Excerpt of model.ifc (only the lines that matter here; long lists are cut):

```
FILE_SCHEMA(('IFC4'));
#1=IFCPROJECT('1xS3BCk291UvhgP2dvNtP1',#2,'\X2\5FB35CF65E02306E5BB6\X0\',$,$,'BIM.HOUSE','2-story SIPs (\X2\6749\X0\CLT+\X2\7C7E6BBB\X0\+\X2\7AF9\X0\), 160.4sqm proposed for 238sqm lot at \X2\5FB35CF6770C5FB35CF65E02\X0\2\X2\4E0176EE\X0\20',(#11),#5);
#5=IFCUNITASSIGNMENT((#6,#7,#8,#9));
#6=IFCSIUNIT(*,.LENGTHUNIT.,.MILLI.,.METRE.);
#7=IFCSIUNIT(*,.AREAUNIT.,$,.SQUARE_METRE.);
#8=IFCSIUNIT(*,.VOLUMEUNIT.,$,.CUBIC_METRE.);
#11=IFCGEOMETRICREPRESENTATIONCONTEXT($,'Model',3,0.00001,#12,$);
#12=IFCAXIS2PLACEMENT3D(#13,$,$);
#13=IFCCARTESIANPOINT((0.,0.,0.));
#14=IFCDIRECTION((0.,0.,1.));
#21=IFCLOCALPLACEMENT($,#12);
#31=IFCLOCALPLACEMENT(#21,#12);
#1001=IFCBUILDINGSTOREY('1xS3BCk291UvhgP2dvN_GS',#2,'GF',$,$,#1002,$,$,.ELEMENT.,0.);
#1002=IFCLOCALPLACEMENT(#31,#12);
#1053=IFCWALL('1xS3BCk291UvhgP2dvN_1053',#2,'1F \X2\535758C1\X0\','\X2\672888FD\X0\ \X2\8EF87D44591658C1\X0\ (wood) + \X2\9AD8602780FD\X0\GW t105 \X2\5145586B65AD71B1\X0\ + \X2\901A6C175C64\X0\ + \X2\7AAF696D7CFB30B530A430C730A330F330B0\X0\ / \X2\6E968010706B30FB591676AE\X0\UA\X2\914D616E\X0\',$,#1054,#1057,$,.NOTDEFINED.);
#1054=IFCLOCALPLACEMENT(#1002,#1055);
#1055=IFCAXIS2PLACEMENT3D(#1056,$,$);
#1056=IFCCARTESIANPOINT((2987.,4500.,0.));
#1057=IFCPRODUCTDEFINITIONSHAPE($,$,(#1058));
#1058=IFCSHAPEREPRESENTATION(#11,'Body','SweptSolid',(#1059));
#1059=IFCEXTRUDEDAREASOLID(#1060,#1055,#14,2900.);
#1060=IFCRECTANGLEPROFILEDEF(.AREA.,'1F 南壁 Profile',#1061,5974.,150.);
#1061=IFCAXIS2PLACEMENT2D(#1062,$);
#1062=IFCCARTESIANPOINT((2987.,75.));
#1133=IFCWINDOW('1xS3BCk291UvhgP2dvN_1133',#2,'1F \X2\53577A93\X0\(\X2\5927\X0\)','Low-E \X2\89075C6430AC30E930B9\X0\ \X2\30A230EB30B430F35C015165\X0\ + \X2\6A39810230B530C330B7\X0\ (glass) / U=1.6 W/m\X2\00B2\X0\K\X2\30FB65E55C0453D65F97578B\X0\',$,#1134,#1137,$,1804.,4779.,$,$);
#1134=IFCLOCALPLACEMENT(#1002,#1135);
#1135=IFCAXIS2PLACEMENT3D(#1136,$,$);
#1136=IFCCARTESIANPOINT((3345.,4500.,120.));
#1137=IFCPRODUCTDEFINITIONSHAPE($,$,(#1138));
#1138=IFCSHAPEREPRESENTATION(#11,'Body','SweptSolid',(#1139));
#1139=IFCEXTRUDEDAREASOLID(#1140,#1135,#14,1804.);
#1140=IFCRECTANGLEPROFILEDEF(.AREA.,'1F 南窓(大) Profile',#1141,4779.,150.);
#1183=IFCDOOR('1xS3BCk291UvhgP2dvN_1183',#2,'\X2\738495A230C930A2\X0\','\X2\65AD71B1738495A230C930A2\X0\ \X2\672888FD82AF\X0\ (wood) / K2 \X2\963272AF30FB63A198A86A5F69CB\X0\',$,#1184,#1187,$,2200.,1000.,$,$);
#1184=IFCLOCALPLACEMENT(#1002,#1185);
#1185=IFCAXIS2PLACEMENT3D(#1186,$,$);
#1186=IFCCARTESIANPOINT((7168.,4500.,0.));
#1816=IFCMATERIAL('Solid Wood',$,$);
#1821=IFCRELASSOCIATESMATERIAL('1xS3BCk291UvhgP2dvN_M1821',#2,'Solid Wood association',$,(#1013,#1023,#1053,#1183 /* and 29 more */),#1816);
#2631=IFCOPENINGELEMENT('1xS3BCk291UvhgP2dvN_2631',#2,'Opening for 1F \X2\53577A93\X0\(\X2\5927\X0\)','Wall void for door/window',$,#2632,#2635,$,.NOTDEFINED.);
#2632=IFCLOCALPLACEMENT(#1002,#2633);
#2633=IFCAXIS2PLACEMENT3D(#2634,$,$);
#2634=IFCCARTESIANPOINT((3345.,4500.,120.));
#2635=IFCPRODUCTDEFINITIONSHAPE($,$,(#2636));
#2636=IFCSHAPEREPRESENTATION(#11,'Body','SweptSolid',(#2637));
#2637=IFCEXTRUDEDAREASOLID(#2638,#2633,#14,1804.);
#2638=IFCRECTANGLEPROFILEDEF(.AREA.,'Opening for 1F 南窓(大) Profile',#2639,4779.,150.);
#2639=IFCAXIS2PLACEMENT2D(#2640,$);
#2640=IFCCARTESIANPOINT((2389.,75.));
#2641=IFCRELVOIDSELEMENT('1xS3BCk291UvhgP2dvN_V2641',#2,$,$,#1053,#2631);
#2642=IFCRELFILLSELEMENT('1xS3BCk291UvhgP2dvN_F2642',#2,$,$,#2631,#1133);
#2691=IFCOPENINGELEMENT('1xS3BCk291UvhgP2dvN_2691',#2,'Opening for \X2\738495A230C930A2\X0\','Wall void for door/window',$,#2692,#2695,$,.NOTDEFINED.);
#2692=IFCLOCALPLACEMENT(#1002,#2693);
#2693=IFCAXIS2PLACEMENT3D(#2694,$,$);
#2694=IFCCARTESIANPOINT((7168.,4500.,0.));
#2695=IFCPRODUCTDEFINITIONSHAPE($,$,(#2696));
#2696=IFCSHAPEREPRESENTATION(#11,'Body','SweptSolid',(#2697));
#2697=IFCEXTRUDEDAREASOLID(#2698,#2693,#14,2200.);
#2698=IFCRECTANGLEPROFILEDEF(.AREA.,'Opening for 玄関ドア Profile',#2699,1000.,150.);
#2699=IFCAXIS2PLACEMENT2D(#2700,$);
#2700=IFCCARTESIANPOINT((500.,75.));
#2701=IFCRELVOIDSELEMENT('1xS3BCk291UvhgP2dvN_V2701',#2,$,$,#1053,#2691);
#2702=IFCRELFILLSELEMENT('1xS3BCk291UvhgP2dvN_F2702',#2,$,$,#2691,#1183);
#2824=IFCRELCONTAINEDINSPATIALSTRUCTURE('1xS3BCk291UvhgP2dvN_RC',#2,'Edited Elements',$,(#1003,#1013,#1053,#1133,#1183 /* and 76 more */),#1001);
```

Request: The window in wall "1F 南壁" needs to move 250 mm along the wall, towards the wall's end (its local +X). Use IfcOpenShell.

```python
import ifcopenshell
import ifcopenshell.api.geometry
import ifcopenshell.util.placement
import ifcopenshell.util.unit

model = ifcopenshell.open("model.ifc")
unit_scale = ifcopenshell.util.unit.calculate_unit_scale(model)

window = model.by_guid("1xS3BCk291UvhgP2dvN_1133")
opening = window.FillsVoids[0].RelatingOpeningElement
wall = opening.VoidsElements[0].RelatingBuildingElement

wall_matrix = ifcopenshell.util.placement.get_local_placement(wall.ObjectPlacement)
shift = wall_matrix[:3, 0] * 0.25 / unit_scale
before = ifcopenshell.util.placement.get_local_placement(window.ObjectPlacement)[:3, 3].copy()

# The window is not placed relative to its opening, so move both.
for product in (opening, window):
    matrix = ifcopenshell.util.placement.get_local_placement(product.ObjectPlacement)
    matrix[:3, 3] += shift
    ifcopenshell.api.geometry.edit_object_placement(model, product=product, matrix=matrix, is_si=False)

after = ifcopenshell.util.placement.get_local_placement(window.ObjectPlacement)[:3, 3]
print("window moved by", (after - before).round(3) + 0.0)

model.write("model-out.ifc")
```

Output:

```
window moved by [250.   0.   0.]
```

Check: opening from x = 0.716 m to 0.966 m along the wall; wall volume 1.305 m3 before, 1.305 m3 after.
